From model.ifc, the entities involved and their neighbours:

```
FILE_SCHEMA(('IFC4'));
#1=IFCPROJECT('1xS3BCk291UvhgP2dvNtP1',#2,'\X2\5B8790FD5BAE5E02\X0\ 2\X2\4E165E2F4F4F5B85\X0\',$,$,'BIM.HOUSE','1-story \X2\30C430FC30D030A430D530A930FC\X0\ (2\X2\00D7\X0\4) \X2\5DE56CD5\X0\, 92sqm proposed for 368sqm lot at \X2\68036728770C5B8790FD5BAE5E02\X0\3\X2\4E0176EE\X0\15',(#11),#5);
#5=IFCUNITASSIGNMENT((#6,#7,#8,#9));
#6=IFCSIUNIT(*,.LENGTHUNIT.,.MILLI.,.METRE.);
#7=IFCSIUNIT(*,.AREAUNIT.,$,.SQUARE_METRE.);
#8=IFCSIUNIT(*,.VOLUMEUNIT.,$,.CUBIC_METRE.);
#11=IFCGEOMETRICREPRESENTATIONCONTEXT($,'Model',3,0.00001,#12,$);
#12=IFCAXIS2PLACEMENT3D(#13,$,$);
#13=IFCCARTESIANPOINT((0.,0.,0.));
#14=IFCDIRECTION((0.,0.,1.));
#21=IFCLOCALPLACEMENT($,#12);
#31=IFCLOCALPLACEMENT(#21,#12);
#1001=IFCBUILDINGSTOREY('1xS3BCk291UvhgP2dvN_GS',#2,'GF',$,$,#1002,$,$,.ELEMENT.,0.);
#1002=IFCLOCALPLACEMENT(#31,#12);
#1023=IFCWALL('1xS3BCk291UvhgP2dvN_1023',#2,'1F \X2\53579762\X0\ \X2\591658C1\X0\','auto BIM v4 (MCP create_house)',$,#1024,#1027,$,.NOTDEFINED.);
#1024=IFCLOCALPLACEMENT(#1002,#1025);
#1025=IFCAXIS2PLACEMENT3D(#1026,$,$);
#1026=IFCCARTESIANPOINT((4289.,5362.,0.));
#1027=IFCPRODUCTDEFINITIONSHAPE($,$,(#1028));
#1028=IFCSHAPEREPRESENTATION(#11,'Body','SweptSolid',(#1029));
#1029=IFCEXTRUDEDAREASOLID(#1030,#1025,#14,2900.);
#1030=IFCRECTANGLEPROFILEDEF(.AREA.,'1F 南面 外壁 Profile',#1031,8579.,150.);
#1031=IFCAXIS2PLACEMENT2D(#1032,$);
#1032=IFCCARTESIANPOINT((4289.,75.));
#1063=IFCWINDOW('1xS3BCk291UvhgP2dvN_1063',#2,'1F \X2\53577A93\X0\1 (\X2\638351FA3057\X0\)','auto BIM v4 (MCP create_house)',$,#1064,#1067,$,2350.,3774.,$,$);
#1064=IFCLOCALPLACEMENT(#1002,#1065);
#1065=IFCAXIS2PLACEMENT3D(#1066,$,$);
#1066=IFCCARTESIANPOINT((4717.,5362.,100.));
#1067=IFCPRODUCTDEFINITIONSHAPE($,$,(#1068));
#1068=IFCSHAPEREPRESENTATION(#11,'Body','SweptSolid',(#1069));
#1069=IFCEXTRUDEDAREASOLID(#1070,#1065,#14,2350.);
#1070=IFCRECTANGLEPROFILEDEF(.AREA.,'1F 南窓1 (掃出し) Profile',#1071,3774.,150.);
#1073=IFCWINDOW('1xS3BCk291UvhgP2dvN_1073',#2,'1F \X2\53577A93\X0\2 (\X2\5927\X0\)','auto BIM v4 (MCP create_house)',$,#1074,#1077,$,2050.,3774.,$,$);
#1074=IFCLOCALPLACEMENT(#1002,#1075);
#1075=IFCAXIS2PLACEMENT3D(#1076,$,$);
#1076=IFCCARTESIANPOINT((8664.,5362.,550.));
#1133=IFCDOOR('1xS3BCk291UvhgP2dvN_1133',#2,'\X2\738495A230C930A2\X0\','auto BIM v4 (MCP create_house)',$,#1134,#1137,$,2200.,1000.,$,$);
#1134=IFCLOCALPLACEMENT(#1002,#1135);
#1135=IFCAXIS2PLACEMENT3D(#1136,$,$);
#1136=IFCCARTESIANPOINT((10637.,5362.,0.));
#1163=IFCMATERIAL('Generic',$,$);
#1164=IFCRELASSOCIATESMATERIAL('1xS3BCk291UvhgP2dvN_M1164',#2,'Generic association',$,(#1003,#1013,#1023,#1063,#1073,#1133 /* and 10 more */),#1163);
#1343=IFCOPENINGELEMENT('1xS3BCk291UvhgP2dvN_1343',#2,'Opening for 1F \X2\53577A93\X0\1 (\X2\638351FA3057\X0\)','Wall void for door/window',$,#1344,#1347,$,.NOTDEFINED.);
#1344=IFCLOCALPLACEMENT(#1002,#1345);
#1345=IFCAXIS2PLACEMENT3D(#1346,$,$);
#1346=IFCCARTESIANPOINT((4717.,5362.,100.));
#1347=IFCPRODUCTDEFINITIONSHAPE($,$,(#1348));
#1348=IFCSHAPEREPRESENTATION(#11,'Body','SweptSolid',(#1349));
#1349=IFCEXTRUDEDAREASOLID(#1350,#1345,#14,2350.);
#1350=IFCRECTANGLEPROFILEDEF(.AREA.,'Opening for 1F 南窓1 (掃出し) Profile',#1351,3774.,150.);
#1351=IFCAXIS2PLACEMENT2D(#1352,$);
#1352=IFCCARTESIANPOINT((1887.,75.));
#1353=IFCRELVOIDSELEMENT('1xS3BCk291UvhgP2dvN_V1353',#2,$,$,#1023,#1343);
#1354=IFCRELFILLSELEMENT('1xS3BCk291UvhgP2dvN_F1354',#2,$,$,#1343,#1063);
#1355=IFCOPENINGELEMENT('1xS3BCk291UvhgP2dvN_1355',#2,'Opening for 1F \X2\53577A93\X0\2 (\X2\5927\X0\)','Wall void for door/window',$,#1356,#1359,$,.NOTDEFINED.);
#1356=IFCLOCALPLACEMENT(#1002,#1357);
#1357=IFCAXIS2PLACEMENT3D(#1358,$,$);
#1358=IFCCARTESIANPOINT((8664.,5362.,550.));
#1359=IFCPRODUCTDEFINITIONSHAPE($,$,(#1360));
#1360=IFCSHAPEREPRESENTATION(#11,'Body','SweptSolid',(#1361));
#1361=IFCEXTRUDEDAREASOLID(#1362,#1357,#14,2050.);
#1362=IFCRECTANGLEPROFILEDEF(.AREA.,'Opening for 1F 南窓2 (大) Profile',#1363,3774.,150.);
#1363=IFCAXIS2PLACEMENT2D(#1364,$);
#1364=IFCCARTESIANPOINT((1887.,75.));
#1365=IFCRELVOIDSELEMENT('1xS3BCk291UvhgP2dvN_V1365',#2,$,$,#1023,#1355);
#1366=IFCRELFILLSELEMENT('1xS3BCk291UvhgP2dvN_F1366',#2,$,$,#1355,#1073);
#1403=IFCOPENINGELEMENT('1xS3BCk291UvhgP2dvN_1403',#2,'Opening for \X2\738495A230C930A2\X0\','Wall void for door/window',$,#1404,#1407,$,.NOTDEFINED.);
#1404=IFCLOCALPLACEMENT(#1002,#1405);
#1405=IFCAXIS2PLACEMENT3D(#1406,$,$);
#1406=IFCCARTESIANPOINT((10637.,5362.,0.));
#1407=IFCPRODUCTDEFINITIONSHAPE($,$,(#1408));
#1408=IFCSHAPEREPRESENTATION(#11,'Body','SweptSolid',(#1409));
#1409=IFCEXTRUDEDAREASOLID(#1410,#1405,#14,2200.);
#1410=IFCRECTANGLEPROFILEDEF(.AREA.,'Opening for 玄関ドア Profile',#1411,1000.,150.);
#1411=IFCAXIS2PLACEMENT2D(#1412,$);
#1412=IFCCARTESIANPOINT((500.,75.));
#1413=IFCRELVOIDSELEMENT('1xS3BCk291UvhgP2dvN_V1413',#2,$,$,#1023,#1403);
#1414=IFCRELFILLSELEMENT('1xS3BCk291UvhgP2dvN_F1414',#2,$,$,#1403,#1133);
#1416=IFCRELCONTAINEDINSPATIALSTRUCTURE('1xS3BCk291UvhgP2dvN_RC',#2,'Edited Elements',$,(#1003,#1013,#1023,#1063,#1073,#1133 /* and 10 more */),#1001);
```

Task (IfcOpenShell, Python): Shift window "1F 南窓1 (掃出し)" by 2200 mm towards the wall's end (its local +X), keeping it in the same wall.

```python
import ifcopenshell
import ifcopenshell.api.geometry
import ifcopenshell.util.placement

model = ifcopenshell.open("model.ifc")

window = model.by_guid("1xS3BCk291UvhgP2dvN_1063")
opening = window.FillsVoids[0].RelatingOpeningElement
wall = opening.VoidsElements[0].RelatingBuildingElement

wall_matrix = ifcopenshell.util.placement.get_local_placement(wall.ObjectPlacement)
shift = wall_matrix[:3, 0] * 2200.0
before = ifcopenshell.util.placement.get_local_placement(window.ObjectPlacement)[:3, 3].copy()

# The window is not placed relative to its opening, so move both.
for product in (opening, window):
    matrix = ifcopenshell.util.placement.get_local_placement(product.ObjectPlacement)
    matrix[:3, 3] += shift
    ifcopenshell.api.geometry.edit_object_placement(model, product=product, matrix=matrix, is_si=False)

after = ifcopenshell.util.placement.get_local_placement(window.ObjectPlacement)[:3, 3]
print("window moved by", (after - before).round(3) + 0.0)

model.write("model_v2.ifc")
```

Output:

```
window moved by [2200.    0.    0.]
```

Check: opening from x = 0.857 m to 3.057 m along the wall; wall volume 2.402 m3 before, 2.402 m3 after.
